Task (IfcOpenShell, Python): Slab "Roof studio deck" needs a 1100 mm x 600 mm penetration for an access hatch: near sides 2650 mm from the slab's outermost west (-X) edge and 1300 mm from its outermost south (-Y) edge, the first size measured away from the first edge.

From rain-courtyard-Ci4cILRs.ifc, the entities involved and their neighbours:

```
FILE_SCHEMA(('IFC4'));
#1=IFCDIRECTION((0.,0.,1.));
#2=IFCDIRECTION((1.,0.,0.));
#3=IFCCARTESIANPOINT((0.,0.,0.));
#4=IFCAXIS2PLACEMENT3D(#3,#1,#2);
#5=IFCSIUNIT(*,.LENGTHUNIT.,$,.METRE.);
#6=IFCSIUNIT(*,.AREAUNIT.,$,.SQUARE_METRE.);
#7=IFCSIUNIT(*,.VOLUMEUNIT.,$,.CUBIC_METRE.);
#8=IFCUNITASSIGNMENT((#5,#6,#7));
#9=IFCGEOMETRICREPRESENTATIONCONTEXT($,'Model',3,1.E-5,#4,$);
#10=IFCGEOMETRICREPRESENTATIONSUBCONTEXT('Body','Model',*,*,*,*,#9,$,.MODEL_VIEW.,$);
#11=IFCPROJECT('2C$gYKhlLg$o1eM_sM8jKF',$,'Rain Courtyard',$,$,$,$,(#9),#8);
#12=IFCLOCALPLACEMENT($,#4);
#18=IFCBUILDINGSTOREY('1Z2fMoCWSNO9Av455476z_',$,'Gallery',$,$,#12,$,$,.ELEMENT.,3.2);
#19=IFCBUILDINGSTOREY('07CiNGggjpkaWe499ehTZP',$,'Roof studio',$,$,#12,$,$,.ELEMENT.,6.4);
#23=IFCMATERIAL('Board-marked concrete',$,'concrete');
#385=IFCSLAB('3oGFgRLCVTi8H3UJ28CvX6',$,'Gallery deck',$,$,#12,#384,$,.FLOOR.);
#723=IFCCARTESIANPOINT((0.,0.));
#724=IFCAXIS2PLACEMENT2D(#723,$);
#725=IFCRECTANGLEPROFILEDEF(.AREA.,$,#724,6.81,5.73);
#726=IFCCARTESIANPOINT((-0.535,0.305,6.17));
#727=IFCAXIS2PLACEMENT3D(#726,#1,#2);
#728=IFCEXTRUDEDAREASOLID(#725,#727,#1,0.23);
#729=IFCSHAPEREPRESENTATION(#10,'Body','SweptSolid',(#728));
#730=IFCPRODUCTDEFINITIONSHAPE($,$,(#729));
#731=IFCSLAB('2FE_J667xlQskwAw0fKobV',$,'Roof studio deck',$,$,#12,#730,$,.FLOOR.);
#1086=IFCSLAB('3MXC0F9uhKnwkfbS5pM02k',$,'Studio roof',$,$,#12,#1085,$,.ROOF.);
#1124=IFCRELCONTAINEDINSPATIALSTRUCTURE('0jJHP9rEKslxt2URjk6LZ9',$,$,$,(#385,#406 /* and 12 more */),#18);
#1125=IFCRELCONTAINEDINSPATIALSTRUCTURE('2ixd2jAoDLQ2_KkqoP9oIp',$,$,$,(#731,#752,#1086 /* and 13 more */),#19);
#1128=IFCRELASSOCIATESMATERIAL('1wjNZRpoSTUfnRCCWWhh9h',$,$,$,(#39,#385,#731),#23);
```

```python
import numpy as np
import ifcopenshell
import ifcopenshell.api.feature
import ifcopenshell.api.geometry
import ifcopenshell.api.root
import ifcopenshell.geom
import ifcopenshell.util.placement
import ifcopenshell.util.representation
import ifcopenshell.util.shape
import ifcopenshell.util.unit

model = ifcopenshell.open("rain-courtyard-Ci4cILRs.ifc")
unit_scale = ifcopenshell.util.unit.calculate_unit_scale(model)
settings = ifcopenshell.geom.settings()


def volume(element):
    """Net volume in cubic metres, openings subtracted."""
    shape = ifcopenshell.geom.create_shape(settings, element)
    return ifcopenshell.util.shape.get_volume(shape.geometry)


slab = model.by_guid("2FE_J667xlQskwAw0fKobV")
before = volume(slab)

# Extent in the slab's own axes, in metres. The edges named are its -X and -Y sides.
slab_shape = ifcopenshell.geom.create_shape(settings, slab)
vertices = ifcopenshell.util.shape.get_vertices(slab_shape.geometry)
x_min, y_min, bottom = vertices.min(axis=0)
top = vertices[:, 2].max()

opening = ifcopenshell.api.root.create_entity(model, ifc_class="IfcOpeningElement", name="Access hatch opening", predefined_type="OPENING")
context = ifcopenshell.util.representation.get_context(model, "Model", "Body", "MODEL_VIEW")
width, depth = 1.1, 0.6
outline = [(0.0, 0.0), (width, 0.0), (width, depth), (0.0, depth), (0.0, 0.0)]
# Overshoot both faces by 50 mm so the cut is clean.
shape = ifcopenshell.api.geometry.add_slab_representation(
    model, context=context, depth=top - bottom + 0.1, polyline=outline
)
ifcopenshell.api.geometry.assign_representation(model, product=opening, representation=shape)

matrix = ifcopenshell.util.placement.get_local_placement(slab.ObjectPlacement)
matrix[:, 3] = matrix @ np.append(np.array([x_min + 2.65, y_min + 1.3, bottom - 0.05]) / unit_scale, 1.0)
ifcopenshell.api.geometry.edit_object_placement(model, product=opening, matrix=matrix, is_si=False)
ifcopenshell.api.feature.add_feature(model, feature=opening, element=slab)

after = volume(slab)

print(f"slab volume {before:.3f} -> {after:.3f} m3")

model.write("rain-courtyard-Ci4cILRs_updated.ifc")
```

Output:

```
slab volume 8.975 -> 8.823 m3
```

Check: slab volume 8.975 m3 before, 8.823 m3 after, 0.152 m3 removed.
